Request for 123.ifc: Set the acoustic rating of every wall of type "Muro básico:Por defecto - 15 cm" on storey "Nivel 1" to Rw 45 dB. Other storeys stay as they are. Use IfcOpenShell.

First a look at what the model holds.

```python
import ifcopenshell
import ifcopenshell.util.element

model = ifcopenshell.open("123.ifc")
print(model.schema)
storey = next(s for s in model.by_type("IfcBuildingStorey") if s.Name == "Nivel 1")
walls = [e for e in ifcopenshell.util.element.get_decomposition(storey) if e.is_a("IfcWall")]
seen = {}
for e in walls:
    element_type = ifcopenshell.util.element.get_type(e)
    key = (element_type.Name if element_type != e and element_type else None, ifcopenshell.util.element.get_pset(e, "Pset_WallCommon", "AcousticRating"))
    seen[key] = seen.get(key, 0) + 1
for (name, value), count in sorted(seen.items(), key=str):
    print(count, "x", name, "|", value)
```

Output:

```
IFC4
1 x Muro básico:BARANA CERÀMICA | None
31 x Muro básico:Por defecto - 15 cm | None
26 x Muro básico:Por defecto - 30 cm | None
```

```python
import ifcopenshell
import ifcopenshell.api.pset
import ifcopenshell.util.element

model = ifcopenshell.open("123.ifc")

storey = next(s for s in model.by_type("IfcBuildingStorey") if s.Name == "Nivel 1")
walls = [e for e in ifcopenshell.util.element.get_decomposition(storey) if e.is_a("IfcWall")]

count = 0
for e in walls:
    element_type = ifcopenshell.util.element.get_type(e)
    if element_type in (None, e) or element_type.Name != "Muro básico:Por defecto - 15 cm":
        continue
    # add_pset returns the element's existing set when there is one.
    pset = ifcopenshell.api.pset.add_pset(model, product=e, name="Pset_WallCommon")
    ifcopenshell.api.pset.edit_pset(model, pset=pset, properties={"AcousticRating": "Rw 45 dB"})
    count += 1

print(count, "walls updated")

model.write("123_edited.ifc")
```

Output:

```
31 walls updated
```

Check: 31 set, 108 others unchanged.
